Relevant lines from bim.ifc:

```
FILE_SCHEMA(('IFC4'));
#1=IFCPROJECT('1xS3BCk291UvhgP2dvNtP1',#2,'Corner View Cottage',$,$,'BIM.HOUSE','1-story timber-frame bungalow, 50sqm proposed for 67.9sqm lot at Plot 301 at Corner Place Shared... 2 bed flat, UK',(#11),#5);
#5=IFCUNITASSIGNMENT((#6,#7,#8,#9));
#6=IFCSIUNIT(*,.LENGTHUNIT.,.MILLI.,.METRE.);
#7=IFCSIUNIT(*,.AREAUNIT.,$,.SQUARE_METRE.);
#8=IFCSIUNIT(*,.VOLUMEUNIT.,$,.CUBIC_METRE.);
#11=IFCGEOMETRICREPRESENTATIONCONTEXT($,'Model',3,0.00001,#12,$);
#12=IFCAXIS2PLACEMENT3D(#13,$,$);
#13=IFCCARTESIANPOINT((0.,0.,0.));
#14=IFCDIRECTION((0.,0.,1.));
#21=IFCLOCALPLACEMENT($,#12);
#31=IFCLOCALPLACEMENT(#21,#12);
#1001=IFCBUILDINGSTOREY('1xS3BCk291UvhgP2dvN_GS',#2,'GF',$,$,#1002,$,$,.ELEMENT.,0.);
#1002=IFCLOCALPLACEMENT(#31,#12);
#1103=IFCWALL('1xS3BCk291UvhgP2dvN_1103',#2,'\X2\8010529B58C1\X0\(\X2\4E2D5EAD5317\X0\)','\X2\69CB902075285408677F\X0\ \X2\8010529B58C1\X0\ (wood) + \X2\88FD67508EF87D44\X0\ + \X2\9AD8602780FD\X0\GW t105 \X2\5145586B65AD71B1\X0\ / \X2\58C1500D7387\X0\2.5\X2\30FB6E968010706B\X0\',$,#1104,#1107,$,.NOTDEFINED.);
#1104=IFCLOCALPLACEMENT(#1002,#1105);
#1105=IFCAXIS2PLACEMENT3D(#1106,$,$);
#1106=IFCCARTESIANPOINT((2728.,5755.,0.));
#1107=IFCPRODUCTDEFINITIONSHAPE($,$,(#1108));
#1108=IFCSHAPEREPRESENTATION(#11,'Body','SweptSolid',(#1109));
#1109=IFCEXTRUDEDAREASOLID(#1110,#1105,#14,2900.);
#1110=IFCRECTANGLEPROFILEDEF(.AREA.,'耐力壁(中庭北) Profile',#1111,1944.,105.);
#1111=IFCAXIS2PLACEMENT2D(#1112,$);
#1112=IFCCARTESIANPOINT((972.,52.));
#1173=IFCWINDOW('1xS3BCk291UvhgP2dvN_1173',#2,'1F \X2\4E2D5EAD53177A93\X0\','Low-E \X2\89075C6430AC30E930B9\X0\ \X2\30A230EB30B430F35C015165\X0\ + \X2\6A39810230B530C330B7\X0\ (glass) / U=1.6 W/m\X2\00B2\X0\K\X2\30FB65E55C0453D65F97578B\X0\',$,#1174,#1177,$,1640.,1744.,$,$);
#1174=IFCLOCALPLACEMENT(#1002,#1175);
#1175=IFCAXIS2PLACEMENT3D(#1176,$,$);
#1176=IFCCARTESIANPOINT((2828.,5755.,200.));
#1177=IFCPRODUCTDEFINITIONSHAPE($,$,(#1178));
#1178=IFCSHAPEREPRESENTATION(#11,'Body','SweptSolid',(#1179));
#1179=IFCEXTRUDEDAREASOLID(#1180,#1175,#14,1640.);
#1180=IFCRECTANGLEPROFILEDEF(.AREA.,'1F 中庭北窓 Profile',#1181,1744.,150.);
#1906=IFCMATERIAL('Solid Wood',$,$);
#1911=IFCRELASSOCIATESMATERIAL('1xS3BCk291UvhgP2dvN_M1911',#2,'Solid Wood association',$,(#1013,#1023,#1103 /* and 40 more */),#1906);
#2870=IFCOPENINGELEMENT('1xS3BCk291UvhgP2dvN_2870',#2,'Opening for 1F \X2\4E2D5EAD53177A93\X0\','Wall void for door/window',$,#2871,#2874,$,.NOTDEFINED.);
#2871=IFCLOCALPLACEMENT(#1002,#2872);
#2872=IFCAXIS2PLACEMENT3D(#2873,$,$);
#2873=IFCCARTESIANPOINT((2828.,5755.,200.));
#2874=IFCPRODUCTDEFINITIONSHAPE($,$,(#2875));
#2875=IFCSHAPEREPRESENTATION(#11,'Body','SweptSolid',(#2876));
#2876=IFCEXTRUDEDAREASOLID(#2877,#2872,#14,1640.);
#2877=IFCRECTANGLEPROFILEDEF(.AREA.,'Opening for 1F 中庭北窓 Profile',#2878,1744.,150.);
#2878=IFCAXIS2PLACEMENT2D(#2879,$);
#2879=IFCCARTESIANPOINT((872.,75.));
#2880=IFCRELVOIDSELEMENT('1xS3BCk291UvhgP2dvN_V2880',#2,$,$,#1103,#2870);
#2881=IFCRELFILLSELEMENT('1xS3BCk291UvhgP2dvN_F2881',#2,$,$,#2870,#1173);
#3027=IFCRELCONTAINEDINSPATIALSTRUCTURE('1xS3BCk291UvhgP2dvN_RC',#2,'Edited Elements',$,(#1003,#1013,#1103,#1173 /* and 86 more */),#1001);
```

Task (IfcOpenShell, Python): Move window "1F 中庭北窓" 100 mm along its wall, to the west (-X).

```python
import ifcopenshell
import ifcopenshell.api.geometry
import ifcopenshell.util.placement

model = ifcopenshell.open("bim.ifc")

window = model.by_id(1173)
opening = window.FillsVoids[0].RelatingOpeningElement
wall = opening.VoidsElements[0].RelatingBuildingElement

wall_matrix = ifcopenshell.util.placement.get_local_placement(wall.ObjectPlacement)
shift = wall_matrix[:3, 0] * -100.0
before = ifcopenshell.util.placement.get_local_placement(window.ObjectPlacement)[:3, 3].copy()

# The window is not placed relative to its opening, so move both.
for product in (opening, window):
    matrix = ifcopenshell.util.placement.get_local_placement(product.ObjectPlacement)
    matrix[:3, 3] += shift
    ifcopenshell.api.geometry.edit_object_placement(model, product=product, matrix=matrix, is_si=False)

after = ifcopenshell.util.placement.get_local_placement(window.ObjectPlacement)[:3, 3]
print("window moved by", (after - before).round(3) + 0.0)

model.write("bim_rev.ifc")
```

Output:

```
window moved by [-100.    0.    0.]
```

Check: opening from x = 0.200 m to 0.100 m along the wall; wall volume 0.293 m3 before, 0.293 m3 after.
